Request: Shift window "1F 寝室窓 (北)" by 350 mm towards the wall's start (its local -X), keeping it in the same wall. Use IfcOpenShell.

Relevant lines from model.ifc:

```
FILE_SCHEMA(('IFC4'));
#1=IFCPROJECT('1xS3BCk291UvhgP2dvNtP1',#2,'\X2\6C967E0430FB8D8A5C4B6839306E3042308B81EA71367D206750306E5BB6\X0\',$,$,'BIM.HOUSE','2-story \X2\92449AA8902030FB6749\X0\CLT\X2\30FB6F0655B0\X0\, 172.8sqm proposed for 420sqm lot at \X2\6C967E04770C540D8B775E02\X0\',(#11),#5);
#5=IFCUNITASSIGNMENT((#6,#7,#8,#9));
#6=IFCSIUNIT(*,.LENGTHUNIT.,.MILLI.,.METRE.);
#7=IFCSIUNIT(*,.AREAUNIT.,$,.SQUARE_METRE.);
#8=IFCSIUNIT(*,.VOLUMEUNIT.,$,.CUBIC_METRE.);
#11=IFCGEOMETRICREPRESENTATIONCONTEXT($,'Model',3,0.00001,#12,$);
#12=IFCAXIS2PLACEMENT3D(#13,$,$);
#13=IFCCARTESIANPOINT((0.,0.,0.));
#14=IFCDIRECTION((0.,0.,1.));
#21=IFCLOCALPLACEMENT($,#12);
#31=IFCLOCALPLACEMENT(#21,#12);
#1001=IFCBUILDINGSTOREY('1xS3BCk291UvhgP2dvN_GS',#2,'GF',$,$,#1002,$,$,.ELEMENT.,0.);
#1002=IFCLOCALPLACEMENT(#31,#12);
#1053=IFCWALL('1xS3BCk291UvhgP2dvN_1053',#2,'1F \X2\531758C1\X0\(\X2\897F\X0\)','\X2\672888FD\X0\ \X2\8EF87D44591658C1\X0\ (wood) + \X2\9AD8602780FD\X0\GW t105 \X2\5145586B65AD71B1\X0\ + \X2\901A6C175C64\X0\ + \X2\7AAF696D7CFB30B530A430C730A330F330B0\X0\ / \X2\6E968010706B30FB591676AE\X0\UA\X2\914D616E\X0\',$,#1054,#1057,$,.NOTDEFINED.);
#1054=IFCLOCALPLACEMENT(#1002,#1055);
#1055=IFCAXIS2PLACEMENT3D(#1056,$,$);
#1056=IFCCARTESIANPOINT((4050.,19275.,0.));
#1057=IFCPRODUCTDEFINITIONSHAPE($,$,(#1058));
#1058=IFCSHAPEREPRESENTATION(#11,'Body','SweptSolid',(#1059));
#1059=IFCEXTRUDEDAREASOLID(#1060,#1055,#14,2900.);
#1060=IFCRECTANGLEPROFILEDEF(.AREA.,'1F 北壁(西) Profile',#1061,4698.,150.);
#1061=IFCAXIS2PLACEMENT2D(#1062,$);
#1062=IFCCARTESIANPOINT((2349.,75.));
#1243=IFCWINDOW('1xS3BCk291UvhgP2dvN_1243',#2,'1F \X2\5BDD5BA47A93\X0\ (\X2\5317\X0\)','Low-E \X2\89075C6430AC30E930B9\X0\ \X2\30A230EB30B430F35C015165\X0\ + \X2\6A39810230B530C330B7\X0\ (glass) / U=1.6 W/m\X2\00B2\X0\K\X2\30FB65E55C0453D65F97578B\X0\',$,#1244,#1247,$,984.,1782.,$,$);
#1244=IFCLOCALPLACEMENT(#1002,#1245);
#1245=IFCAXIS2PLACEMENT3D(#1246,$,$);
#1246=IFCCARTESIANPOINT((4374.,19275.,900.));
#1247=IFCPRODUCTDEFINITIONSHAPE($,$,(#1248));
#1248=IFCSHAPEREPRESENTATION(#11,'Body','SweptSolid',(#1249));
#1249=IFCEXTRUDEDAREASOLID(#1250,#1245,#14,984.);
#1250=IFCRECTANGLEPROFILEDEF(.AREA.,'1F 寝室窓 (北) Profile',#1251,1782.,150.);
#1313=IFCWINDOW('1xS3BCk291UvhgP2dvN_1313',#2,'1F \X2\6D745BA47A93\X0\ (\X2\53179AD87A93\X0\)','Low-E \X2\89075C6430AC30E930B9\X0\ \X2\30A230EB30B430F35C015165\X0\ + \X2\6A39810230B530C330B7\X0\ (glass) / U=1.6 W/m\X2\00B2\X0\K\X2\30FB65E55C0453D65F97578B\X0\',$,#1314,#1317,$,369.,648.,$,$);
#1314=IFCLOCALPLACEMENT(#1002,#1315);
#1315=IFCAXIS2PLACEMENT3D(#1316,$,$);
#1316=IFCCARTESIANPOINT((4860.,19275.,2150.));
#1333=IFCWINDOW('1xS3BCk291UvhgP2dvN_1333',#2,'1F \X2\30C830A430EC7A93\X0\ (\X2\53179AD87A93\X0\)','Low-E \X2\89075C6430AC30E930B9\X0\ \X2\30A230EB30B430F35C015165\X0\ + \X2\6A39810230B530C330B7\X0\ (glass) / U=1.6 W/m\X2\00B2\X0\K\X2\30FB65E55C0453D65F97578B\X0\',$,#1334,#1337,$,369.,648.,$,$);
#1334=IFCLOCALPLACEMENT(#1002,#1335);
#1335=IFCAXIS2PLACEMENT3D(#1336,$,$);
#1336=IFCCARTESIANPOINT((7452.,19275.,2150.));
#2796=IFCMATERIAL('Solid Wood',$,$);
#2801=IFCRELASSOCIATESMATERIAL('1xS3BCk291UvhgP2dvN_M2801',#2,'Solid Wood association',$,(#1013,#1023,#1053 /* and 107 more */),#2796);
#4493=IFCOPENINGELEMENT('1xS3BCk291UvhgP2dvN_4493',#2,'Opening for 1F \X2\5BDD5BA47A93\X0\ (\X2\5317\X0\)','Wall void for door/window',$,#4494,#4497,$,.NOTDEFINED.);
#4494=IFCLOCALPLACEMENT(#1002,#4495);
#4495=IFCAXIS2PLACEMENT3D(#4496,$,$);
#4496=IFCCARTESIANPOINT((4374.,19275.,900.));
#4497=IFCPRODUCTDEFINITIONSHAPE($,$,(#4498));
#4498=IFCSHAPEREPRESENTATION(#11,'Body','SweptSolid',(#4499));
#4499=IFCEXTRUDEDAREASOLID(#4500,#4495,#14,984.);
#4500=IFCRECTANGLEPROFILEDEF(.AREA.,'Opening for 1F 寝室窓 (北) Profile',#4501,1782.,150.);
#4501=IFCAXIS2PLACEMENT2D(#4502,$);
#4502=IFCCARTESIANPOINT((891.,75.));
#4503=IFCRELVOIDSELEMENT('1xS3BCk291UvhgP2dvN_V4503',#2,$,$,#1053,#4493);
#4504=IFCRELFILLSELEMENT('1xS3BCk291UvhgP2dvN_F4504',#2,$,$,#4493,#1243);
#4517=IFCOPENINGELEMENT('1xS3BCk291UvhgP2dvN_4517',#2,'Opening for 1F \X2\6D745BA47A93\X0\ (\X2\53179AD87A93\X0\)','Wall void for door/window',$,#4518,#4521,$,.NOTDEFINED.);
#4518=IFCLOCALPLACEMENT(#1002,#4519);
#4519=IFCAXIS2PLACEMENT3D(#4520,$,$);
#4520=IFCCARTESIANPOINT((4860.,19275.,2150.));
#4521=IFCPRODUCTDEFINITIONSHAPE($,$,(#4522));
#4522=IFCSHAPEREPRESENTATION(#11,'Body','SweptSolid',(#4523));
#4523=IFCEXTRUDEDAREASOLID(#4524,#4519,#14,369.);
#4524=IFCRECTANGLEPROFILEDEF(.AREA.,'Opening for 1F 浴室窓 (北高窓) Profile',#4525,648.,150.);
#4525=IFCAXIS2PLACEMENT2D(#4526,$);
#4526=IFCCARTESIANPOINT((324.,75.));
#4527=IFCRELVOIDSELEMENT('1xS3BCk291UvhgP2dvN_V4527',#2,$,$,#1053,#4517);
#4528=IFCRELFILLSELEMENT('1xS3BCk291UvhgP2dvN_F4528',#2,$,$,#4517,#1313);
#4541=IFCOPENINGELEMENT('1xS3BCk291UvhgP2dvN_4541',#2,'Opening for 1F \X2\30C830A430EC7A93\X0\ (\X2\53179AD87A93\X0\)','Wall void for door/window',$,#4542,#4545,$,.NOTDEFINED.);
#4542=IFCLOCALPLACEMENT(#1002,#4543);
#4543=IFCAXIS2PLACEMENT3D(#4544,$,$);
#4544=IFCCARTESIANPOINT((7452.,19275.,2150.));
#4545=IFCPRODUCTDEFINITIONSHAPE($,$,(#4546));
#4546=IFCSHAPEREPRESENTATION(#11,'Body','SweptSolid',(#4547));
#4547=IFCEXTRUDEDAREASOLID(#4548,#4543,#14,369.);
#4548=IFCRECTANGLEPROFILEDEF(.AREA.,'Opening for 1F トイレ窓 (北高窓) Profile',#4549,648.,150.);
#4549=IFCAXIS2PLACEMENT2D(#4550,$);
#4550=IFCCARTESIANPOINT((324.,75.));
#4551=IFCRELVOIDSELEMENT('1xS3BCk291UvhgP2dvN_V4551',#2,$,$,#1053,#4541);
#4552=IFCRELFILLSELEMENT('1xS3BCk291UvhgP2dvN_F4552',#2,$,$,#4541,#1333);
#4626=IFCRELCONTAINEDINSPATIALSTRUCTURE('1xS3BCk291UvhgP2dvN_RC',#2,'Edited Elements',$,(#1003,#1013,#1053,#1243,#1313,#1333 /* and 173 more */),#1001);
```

```python
import ifcopenshell
import ifcopenshell.api.geometry
import ifcopenshell.util.placement
import ifcopenshell.util.unit

model = ifcopenshell.open("model.ifc")
unit_scale = ifcopenshell.util.unit.calculate_unit_scale(model)

window = model.by_guid("1xS3BCk291UvhgP2dvN_1243")
opening = window.FillsVoids[0].RelatingOpeningElement
wall = opening.VoidsElements[0].RelatingBuildingElement

wall_matrix = ifcopenshell.util.placement.get_local_placement(wall.ObjectPlacement)
shift = wall_matrix[:3, 0] * -0.35 / unit_scale
before = ifcopenshell.util.placement.get_local_placement(window.ObjectPlacement)[:3, 3].copy()

# The window is not placed relative to its opening, so move both.
for product in (opening, window):
    matrix = ifcopenshell.util.placement.get_local_placement(product.ObjectPlacement)
    matrix[:3, 3] += shift
    ifcopenshell.api.geometry.edit_object_placement(model, product=product, matrix=matrix, is_si=False)

after = ifcopenshell.util.placement.get_local_placement(window.ObjectPlacement)[:3, 3]
print("window moved by", (after - before).round(3) + 0.0)

model.write("model_updated.ifc")
```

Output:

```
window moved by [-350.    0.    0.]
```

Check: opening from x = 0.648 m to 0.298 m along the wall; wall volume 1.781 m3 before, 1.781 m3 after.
